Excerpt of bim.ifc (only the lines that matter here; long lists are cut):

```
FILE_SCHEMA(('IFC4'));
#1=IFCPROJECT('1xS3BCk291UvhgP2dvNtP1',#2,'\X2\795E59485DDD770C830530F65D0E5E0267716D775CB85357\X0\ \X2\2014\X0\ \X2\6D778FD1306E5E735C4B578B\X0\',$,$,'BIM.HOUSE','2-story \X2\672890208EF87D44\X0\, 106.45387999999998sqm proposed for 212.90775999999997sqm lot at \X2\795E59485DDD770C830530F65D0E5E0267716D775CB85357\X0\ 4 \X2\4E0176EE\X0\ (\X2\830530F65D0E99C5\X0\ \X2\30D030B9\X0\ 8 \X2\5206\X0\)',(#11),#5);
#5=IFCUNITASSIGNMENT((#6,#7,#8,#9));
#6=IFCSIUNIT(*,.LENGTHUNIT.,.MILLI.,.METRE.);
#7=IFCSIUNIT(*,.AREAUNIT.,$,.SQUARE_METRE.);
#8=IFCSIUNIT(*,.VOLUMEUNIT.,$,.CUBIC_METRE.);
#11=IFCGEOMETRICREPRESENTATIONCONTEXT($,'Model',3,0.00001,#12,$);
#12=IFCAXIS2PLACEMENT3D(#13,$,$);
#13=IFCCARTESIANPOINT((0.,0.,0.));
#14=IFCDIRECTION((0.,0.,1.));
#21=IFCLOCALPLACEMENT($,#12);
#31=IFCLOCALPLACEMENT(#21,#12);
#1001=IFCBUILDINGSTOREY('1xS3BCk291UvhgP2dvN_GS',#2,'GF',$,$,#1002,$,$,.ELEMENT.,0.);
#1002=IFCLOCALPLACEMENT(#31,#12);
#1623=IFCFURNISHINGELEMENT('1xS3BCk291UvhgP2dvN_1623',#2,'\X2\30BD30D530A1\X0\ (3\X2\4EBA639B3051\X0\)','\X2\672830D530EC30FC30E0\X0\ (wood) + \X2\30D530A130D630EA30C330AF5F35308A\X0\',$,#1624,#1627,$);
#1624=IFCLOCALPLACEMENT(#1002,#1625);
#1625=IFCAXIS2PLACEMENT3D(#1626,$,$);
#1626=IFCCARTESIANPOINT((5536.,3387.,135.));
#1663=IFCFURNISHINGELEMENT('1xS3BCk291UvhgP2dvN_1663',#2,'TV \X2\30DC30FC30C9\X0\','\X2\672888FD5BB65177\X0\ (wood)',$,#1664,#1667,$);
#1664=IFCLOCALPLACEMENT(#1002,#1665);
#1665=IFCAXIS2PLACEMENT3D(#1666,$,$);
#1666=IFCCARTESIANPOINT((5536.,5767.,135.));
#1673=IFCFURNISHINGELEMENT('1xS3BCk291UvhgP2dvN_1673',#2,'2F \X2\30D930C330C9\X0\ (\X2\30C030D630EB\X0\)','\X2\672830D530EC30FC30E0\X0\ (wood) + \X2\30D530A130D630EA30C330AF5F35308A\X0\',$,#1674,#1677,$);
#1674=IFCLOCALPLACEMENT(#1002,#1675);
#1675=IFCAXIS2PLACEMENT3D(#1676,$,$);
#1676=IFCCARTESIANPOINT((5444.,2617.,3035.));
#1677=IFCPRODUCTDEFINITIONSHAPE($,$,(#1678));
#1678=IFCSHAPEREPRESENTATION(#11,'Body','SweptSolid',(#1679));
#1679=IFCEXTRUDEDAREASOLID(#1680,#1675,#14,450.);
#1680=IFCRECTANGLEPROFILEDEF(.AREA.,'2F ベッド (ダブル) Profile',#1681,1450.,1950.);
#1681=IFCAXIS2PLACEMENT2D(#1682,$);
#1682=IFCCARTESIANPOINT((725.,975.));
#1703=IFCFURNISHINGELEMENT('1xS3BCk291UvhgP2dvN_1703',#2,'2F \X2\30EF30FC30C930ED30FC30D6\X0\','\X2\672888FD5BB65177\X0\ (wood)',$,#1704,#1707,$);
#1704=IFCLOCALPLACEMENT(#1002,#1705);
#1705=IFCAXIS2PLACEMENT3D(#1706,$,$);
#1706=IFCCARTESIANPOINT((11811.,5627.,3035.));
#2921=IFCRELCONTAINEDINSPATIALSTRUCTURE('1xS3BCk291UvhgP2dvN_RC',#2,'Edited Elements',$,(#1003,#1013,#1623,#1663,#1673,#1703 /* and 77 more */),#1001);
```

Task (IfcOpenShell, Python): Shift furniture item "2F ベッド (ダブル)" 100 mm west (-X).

```python
import ifcopenshell
import ifcopenshell.api.geometry
import ifcopenshell.util.placement

model = ifcopenshell.open("bim.ifc")

item = model.by_id(1673)
matrix = ifcopenshell.util.placement.get_local_placement(item.ObjectPlacement)
matrix[0, 3] -= 100.0
ifcopenshell.api.geometry.edit_object_placement(model, product=item, matrix=matrix, is_si=False)

print(ifcopenshell.util.placement.get_local_placement(item.ObjectPlacement).round(3) + 0.0)

model.write("bim_rev.ifc")
```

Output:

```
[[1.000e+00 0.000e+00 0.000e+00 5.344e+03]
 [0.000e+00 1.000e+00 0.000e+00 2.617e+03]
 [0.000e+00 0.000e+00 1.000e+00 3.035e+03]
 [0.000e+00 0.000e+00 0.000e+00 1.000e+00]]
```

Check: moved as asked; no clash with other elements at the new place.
